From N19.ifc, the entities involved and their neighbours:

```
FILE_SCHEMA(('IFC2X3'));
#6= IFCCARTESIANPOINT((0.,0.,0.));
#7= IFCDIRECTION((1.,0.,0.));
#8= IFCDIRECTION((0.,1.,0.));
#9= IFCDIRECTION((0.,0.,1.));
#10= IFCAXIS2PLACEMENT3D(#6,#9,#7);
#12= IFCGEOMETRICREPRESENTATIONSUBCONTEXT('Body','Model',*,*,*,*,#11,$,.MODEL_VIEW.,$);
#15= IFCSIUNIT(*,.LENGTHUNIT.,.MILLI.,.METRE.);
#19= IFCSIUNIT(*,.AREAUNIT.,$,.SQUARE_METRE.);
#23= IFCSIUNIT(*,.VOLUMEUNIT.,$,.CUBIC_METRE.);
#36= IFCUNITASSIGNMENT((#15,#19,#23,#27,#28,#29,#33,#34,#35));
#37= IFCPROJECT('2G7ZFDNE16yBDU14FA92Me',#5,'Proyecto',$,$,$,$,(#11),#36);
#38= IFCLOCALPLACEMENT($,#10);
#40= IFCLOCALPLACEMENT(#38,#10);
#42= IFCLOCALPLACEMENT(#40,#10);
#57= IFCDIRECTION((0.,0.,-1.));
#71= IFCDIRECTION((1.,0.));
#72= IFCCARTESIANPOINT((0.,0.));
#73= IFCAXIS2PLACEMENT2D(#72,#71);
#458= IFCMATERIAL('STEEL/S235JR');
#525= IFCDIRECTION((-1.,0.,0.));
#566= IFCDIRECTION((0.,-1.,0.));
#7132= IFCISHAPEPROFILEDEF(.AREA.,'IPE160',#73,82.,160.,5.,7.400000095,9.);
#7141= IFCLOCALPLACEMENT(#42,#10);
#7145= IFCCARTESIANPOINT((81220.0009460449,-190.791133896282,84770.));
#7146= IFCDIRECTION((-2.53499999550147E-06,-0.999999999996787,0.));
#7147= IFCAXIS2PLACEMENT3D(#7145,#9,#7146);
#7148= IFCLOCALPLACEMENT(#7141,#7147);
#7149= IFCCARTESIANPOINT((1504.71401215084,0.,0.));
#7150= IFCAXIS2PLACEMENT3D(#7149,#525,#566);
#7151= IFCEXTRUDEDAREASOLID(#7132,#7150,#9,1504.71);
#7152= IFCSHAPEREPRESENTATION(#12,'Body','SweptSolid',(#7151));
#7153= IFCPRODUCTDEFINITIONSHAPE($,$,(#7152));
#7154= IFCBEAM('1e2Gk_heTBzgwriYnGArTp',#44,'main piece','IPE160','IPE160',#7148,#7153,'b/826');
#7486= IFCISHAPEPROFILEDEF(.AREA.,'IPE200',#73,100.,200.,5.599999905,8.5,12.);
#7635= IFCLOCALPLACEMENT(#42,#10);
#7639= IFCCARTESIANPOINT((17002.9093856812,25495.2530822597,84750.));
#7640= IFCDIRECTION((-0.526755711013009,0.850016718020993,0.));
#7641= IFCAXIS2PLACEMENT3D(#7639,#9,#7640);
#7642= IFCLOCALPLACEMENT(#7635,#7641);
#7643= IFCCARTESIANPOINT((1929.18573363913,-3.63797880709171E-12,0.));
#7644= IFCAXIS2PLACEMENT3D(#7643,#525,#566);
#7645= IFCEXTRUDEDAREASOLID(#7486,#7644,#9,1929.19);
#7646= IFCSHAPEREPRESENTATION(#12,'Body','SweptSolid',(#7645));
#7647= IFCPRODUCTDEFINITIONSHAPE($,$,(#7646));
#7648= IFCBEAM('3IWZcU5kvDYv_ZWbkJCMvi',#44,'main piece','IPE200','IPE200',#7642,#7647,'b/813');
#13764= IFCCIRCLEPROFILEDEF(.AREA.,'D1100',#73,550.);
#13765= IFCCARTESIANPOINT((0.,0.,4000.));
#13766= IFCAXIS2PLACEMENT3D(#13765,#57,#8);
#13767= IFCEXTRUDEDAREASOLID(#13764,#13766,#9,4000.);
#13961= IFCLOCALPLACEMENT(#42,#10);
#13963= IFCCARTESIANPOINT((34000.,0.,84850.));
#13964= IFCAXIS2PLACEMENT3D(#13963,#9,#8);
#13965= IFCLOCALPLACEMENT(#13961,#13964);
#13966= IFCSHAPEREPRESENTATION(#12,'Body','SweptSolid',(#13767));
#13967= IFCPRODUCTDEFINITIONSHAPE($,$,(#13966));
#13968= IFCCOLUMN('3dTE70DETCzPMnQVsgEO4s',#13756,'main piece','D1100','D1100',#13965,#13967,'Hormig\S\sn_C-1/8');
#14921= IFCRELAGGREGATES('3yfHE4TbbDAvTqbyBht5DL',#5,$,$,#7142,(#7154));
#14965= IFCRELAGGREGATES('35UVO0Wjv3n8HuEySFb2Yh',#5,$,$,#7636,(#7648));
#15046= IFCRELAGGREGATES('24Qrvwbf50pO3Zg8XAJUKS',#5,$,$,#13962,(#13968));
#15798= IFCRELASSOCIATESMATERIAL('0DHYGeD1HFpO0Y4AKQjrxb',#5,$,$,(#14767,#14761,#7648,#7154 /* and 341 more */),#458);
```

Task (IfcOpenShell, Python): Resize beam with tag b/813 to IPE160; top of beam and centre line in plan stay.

```python
import ifcopenshell
import ifcopenshell.util.element
import ifcopenshell.util.representation

model = ifcopenshell.open("N19.ifc")

member = model.by_guid("3IWZcU5kvDYv_ZWbkJCMvi")
source = next(p for p in model.by_type("IfcIShapeProfileDef") if p.ProfileName == "IPE160")

body = ifcopenshell.util.representation.get_representation(member, "Model", "Body")
solid = body.Items[0]
old_profile = solid.SweptArea

# Copy the section's sizes but keep this member's own profile position.
profile = ifcopenshell.util.element.copy(model, source)
# Profiles are centred, so shift by half the change in depth to hold the top.
shift = (old_profile.OverallDepth - profile.OverallDepth) / 2
x, y = old_profile.Position.Location.Coordinates
up = (0.0, 1.0)  # upwards, in the solid's own plane
location = model.createIfcCartesianPoint((x + up[0] * shift, y + up[1] * shift))
profile.Position = model.createIfcAxis2Placement2D(location, old_profile.Position.RefDirection)
solid.SweptArea = profile
if not model.get_total_inverses(old_profile):
    ifcopenshell.util.element.remove_deep2(model, old_profile)
member.Description = member.Description.replace("IPE200", "IPE160")
member.ObjectType = member.ObjectType.replace("IPE200", "IPE160")

print(solid.SweptArea)

model.write("N19-out.ifc")
```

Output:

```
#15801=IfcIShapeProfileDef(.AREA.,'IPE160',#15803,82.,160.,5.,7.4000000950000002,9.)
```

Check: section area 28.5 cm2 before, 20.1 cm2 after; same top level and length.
